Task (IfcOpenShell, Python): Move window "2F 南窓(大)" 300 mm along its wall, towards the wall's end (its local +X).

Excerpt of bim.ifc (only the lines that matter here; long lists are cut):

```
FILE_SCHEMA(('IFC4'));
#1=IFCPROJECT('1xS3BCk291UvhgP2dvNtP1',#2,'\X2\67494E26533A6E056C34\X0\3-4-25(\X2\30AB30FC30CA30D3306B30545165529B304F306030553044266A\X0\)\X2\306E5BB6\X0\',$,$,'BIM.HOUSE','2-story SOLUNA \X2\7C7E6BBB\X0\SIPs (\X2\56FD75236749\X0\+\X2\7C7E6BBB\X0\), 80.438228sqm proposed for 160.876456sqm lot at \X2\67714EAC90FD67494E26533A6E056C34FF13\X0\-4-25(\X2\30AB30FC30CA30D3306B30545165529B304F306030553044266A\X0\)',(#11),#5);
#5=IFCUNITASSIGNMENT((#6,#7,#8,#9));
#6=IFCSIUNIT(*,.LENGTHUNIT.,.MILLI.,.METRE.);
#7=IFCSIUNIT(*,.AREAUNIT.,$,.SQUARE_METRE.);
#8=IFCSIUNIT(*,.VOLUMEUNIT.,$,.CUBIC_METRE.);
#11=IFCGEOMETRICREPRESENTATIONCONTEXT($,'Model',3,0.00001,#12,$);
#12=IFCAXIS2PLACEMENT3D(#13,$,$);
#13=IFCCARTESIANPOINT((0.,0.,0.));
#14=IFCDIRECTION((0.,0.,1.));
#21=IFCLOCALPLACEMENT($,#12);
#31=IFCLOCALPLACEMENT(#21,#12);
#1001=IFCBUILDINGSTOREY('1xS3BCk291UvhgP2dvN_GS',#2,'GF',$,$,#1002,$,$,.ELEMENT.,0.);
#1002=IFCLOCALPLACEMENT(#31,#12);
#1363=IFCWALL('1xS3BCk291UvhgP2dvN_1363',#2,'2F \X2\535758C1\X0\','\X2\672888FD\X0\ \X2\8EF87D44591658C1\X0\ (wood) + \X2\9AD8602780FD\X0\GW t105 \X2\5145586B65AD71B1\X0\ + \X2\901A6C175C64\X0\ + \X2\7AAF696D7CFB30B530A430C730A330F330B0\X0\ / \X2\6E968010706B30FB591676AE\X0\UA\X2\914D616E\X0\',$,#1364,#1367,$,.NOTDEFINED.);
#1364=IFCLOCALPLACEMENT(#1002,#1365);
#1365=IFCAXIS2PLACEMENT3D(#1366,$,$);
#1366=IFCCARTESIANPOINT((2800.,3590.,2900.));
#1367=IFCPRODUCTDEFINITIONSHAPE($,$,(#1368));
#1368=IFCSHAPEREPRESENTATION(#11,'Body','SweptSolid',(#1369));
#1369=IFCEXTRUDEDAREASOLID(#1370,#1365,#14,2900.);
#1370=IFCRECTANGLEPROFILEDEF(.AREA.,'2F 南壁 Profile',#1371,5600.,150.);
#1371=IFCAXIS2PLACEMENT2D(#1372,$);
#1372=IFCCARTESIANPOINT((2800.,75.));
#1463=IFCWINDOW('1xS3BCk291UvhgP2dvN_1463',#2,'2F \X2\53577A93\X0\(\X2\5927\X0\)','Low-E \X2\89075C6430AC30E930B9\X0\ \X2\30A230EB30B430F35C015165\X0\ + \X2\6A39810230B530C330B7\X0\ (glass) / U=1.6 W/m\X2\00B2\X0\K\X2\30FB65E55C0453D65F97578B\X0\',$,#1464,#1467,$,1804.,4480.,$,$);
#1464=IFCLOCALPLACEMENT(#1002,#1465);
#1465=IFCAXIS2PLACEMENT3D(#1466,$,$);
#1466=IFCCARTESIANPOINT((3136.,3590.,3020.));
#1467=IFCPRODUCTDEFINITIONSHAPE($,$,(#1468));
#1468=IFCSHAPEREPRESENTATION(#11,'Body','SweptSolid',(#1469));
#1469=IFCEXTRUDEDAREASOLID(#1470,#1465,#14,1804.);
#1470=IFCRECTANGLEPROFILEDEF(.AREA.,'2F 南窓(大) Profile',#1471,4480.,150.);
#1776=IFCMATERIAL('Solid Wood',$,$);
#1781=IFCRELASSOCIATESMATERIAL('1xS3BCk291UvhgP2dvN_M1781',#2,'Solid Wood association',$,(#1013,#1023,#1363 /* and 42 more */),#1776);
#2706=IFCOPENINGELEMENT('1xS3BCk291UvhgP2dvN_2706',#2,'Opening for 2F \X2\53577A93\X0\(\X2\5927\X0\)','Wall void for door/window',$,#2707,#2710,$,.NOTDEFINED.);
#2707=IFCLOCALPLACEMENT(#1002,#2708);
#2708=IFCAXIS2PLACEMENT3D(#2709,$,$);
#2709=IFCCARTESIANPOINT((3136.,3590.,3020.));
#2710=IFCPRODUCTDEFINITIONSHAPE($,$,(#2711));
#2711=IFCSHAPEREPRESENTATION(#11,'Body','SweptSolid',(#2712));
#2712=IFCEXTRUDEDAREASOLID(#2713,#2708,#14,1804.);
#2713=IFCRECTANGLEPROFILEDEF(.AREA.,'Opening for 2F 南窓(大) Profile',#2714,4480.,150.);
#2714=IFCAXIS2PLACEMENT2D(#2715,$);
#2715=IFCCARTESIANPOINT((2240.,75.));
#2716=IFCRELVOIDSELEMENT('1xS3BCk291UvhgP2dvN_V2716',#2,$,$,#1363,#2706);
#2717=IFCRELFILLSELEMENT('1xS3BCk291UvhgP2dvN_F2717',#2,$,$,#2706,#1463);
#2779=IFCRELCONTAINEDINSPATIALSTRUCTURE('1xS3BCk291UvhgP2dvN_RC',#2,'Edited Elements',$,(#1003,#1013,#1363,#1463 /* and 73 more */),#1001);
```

```python
import ifcopenshell
import ifcopenshell.api.geometry
import ifcopenshell.util.placement

model = ifcopenshell.open("bim.ifc")

window = model.by_id(1463)
opening = window.FillsVoids[0].RelatingOpeningElement
wall = opening.VoidsElements[0].RelatingBuildingElement

wall_matrix = ifcopenshell.util.placement.get_local_placement(wall.ObjectPlacement)
shift = wall_matrix[:3, 0] * 300.0
before = ifcopenshell.util.placement.get_local_placement(window.ObjectPlacement)[:3, 3].copy()

# The window is not placed relative to its opening, so move both.
for product in (opening, window):
    matrix = ifcopenshell.util.placement.get_local_placement(product.ObjectPlacement)
    matrix[:3, 3] += shift
    ifcopenshell.api.geometry.edit_object_placement(model, product=product, matrix=matrix, is_si=False)

after = ifcopenshell.util.placement.get_local_placement(window.ObjectPlacement)[:3, 3]
print("window moved by", (after - before).round(3) + 0.0)

model.write("bim_updated.ifc")
```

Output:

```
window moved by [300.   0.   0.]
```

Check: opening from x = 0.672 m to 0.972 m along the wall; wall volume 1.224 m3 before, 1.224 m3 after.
